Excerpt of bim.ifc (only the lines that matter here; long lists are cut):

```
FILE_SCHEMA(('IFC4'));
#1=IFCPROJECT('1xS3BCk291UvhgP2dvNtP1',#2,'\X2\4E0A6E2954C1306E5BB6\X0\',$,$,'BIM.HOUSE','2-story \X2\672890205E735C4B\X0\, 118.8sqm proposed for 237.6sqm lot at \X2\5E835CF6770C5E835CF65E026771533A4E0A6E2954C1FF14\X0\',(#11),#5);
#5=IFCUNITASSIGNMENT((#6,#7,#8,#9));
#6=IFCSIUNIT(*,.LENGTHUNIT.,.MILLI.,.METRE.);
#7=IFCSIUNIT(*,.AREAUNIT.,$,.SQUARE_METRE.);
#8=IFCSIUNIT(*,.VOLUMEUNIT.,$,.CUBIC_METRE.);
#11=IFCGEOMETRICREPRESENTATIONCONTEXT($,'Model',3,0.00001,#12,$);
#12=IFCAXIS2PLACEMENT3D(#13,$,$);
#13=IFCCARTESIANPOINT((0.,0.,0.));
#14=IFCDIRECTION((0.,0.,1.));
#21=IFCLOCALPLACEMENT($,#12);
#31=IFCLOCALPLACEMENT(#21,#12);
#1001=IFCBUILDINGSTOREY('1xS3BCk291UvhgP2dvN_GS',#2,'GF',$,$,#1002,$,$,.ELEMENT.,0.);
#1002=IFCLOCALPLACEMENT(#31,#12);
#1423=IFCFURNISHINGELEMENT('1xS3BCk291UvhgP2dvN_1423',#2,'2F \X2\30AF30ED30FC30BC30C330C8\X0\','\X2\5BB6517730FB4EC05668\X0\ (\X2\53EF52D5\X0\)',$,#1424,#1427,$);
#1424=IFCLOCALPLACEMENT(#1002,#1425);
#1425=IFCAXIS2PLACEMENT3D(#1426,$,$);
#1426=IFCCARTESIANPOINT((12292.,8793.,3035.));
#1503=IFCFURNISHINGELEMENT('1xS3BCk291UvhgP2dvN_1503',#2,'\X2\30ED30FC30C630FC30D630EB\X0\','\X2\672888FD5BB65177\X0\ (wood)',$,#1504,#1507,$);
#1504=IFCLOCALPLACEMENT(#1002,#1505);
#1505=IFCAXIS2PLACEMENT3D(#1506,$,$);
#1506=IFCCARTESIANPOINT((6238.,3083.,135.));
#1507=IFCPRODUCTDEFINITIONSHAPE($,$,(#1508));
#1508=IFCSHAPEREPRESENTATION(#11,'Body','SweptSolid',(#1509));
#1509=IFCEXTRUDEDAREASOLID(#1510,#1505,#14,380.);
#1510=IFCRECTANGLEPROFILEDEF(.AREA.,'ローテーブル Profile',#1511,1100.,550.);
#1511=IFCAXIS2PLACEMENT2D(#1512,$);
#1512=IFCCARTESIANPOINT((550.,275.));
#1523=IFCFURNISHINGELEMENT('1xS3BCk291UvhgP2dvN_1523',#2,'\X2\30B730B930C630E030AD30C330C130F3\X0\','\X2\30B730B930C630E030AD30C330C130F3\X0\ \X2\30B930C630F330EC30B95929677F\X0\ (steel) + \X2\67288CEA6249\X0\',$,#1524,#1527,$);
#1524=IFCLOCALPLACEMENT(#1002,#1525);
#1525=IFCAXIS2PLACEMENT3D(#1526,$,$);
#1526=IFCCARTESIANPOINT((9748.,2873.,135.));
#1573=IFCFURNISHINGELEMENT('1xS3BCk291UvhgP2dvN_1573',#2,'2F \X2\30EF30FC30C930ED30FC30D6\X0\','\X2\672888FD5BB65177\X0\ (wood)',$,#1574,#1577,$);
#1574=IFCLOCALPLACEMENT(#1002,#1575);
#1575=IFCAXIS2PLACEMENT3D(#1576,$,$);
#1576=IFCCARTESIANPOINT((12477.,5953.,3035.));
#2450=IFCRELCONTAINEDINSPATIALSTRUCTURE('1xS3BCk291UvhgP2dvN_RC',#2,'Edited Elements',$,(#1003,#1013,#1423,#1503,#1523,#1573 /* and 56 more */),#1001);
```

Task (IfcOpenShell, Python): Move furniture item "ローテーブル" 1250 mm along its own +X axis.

```python
import ifcopenshell
import ifcopenshell.api.geometry
import ifcopenshell.util.placement

model = ifcopenshell.open("bim.ifc")

item = model.by_guid("1xS3BCk291UvhgP2dvN_1503")
matrix = ifcopenshell.util.placement.get_local_placement(item.ObjectPlacement)
matrix[:3, 3] += matrix[:3, 0] * 1250.0
ifcopenshell.api.geometry.edit_object_placement(model, product=item, matrix=matrix, is_si=False)

print(ifcopenshell.util.placement.get_local_placement(item.ObjectPlacement).round(3) + 0.0)

model.write("bim_v2.ifc")
```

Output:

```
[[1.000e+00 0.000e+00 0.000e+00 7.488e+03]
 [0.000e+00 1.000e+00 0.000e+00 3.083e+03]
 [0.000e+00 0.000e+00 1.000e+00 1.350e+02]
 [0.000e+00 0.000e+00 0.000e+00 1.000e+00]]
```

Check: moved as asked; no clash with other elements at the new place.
